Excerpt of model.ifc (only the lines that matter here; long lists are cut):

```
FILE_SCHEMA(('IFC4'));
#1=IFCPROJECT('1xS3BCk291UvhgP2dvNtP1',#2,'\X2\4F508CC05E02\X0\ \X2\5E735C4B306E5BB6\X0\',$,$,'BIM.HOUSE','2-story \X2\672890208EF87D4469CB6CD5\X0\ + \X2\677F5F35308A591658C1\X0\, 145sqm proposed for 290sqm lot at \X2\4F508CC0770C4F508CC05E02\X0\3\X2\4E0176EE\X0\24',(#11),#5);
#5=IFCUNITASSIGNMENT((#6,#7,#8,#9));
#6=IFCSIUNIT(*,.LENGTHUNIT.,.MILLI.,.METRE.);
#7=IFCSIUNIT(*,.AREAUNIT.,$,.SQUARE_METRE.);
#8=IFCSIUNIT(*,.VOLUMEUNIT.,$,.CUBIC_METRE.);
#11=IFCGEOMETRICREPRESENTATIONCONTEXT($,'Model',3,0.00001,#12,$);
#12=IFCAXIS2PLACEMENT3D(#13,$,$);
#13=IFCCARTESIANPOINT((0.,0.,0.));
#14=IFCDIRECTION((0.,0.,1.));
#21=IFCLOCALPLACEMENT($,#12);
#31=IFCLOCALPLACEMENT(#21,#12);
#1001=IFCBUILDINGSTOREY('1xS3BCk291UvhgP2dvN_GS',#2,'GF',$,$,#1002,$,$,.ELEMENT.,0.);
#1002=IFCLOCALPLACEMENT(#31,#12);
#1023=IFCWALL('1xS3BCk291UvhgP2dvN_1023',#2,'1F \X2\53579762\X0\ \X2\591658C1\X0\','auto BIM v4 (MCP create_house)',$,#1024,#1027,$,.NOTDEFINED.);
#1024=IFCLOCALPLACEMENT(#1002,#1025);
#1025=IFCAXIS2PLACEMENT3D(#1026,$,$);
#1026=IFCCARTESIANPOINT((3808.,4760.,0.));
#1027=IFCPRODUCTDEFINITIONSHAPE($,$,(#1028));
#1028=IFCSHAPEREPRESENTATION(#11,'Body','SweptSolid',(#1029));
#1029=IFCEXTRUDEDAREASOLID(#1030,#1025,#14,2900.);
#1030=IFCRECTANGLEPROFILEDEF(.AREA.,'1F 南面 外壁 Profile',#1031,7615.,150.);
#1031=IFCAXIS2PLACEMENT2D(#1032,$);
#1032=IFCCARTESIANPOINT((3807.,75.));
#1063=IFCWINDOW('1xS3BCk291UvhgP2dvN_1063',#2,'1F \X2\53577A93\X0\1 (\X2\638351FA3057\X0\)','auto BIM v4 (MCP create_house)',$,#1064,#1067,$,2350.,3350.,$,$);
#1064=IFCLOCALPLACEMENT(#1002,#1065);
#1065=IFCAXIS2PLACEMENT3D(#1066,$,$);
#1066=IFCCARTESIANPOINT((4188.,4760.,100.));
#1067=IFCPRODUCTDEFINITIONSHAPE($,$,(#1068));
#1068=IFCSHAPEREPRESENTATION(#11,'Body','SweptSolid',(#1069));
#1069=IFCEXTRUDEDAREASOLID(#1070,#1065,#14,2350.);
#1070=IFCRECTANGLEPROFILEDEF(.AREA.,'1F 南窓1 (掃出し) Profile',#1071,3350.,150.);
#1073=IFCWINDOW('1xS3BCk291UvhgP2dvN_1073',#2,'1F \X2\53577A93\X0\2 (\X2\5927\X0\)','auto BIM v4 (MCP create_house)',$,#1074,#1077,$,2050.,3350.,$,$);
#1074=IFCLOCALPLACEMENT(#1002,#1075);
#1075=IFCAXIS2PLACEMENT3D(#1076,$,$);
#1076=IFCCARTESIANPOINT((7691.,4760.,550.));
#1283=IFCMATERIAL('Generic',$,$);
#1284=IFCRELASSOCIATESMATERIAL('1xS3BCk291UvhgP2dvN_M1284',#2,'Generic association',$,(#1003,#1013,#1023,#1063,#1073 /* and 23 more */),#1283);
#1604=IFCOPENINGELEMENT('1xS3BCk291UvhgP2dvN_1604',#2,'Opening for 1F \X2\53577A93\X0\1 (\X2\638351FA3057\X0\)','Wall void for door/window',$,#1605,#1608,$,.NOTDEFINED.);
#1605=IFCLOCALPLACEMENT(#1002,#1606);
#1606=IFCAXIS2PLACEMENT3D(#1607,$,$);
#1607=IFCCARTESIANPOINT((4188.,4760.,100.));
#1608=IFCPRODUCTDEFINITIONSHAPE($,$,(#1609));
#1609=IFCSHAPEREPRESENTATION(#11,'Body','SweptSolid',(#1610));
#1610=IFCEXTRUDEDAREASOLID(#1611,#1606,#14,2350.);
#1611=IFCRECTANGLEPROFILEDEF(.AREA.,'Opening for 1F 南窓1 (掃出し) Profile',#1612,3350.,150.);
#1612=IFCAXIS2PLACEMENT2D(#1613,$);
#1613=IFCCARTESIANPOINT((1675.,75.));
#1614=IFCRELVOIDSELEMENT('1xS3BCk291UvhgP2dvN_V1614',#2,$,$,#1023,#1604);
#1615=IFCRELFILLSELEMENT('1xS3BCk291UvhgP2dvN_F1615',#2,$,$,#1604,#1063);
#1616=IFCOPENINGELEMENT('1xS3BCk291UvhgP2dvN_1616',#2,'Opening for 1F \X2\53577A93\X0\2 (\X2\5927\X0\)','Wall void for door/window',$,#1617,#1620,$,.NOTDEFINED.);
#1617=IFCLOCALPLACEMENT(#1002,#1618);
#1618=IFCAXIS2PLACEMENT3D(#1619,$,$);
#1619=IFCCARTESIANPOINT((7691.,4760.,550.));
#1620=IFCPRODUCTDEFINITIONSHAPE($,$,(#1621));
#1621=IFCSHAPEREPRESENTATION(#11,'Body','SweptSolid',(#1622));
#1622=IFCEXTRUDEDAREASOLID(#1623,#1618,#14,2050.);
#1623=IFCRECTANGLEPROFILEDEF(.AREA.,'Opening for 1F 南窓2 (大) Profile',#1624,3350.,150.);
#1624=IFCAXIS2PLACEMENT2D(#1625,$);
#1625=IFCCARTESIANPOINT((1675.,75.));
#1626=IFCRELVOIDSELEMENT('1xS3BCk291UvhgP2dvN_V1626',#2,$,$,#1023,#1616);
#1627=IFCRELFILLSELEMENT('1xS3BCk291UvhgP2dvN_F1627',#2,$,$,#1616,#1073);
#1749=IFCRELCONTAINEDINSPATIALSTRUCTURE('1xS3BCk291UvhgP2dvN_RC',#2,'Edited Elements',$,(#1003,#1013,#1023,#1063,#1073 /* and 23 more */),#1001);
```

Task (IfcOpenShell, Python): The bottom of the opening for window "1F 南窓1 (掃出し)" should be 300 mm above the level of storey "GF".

```python
import numpy as np
import ifcopenshell
import ifcopenshell.api.geometry
import ifcopenshell.geom
import ifcopenshell.util.element
import ifcopenshell.util.placement
import ifcopenshell.util.shape
import ifcopenshell.util.unit

model = ifcopenshell.open("model.ifc")
unit_scale = ifcopenshell.util.unit.calculate_unit_scale(model)

window = model.by_guid("1xS3BCk291UvhgP2dvN_1063")
opening = window.FillsVoids[0].RelatingOpeningElement
storey = ifcopenshell.util.element.get_container(window, ifc_class="IfcBuildingStorey")
level = ifcopenshell.util.placement.get_local_placement(storey.ObjectPlacement)[2, 3]

# The opening's origin need not be at the sill, so measure its lowest point.
shape = ifcopenshell.geom.create_shape(ifcopenshell.geom.settings(), opening)
bottom = ifcopenshell.util.shape.get_shape_bottom_elevation(shape, shape.geometry) / unit_scale
dz = level + 300.0 - bottom

shift = np.array([0.0, 0.0, dz])
# The window is not placed relative to its opening, so move both.
for product in (opening, window):
    matrix = ifcopenshell.util.placement.get_local_placement(product.ObjectPlacement)
    matrix[:3, 3] += shift
    ifcopenshell.api.geometry.edit_object_placement(model, product=product, matrix=matrix, is_si=False)

print(f"moved by {dz * unit_scale:+.3f} m")

model.write("model_edited.ifc")
```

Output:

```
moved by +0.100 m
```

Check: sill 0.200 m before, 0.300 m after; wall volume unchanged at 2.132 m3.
